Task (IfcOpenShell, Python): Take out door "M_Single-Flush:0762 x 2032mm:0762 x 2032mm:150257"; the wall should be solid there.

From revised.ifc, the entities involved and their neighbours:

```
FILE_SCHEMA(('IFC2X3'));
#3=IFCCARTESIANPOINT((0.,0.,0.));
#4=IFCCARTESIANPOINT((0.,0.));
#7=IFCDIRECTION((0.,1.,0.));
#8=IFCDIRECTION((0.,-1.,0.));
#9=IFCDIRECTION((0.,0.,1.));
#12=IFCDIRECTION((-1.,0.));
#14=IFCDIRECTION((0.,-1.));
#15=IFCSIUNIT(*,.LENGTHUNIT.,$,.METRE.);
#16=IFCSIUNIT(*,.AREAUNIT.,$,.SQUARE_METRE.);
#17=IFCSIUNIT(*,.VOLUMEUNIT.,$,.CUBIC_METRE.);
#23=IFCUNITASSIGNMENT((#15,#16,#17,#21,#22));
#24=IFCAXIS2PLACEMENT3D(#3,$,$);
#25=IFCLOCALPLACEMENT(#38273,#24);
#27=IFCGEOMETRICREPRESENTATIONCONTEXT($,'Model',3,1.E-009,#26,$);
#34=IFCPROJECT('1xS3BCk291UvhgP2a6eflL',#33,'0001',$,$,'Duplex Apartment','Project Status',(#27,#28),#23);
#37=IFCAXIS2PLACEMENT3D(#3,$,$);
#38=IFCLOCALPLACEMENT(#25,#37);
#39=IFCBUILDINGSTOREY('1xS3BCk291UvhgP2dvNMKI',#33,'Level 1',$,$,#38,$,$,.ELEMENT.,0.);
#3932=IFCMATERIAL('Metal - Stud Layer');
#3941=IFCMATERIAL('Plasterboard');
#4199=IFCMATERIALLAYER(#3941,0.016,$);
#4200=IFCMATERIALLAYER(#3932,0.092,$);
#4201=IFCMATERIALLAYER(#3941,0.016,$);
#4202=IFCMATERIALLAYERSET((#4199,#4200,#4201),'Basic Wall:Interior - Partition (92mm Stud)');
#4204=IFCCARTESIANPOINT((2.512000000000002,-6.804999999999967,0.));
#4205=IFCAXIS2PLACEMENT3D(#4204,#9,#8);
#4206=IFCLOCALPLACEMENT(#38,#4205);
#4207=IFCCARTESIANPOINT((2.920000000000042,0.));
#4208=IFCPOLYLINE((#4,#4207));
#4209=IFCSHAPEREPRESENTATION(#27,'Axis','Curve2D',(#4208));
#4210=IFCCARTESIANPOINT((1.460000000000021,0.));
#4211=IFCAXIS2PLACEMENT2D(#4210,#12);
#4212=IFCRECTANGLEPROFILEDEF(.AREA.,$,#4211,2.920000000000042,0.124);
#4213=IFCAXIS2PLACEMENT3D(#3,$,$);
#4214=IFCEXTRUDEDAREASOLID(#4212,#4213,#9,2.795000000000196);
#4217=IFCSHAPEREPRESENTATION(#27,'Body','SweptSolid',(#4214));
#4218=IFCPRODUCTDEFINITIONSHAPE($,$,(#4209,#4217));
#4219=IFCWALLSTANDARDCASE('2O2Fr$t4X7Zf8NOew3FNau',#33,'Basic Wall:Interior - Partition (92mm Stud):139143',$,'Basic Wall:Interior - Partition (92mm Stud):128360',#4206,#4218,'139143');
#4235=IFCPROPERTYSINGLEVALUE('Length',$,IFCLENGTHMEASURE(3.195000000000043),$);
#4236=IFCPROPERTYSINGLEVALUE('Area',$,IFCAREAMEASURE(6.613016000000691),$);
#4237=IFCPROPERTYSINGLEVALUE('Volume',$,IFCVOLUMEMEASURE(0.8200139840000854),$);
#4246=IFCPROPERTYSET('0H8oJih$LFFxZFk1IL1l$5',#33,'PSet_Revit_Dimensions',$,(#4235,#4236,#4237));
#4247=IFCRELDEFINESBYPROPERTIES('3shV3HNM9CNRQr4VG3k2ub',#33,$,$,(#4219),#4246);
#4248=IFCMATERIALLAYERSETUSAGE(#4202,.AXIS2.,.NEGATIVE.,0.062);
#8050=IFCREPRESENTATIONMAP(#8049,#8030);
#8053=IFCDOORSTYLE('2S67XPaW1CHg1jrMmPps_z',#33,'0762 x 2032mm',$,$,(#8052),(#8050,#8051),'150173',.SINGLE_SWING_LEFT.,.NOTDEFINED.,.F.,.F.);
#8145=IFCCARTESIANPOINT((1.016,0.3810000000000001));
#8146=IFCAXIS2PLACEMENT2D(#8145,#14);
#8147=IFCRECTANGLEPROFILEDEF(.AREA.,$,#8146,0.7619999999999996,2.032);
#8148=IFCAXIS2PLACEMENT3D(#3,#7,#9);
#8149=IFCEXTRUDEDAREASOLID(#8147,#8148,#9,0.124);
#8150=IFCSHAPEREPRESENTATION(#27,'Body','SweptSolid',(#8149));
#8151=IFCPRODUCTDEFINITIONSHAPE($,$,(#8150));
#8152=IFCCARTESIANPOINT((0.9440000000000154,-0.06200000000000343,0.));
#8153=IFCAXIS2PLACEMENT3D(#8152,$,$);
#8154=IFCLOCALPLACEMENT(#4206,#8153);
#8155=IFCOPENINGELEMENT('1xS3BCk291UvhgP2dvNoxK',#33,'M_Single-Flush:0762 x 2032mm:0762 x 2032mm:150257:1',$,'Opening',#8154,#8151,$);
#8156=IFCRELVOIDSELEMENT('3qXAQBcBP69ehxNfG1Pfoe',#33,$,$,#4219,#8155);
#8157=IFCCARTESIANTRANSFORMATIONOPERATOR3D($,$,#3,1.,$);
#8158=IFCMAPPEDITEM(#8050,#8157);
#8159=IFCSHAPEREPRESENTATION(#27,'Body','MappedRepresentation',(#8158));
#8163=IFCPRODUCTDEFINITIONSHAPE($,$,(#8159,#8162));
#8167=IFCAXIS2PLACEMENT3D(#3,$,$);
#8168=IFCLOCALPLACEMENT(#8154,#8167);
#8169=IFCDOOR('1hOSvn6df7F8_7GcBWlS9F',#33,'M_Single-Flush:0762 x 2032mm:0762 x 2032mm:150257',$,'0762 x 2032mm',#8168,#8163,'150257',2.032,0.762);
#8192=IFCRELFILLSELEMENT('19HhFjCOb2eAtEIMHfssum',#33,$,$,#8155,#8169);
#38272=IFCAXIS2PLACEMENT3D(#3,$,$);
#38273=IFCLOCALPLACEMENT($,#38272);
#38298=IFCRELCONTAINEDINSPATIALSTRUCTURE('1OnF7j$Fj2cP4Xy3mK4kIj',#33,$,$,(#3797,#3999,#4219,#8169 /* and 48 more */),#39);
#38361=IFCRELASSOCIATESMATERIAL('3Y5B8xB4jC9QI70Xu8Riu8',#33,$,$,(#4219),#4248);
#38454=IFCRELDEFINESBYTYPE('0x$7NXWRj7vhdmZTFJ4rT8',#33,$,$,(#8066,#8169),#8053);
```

```python
import ifcopenshell
import ifcopenshell.api.feature
import ifcopenshell.api.pset
import ifcopenshell.api.root
import ifcopenshell.geom
import ifcopenshell.util.element
import ifcopenshell.util.shape
import ifcopenshell.util.unit

model = ifcopenshell.open("revised.ifc")
area_scale = ifcopenshell.util.unit.calculate_unit_scale(model, "AREAUNIT")
volume_scale = ifcopenshell.util.unit.calculate_unit_scale(model, "VOLUMEUNIT")
settings = ifcopenshell.geom.settings()


def volume(element):
    """Net volume in cubic metres, openings subtracted."""
    shape = ifcopenshell.geom.create_shape(settings, element)
    return ifcopenshell.util.shape.get_volume(shape.geometry)


door = model.by_guid("1hOSvn6df7F8_7GcBWlS9F")
opening = door.FillsVoids[0].RelatingOpeningElement
wall = opening.VoidsElements[0].RelatingBuildingElement
before = volume(wall)

ifcopenshell.api.root.remove_product(model, product=door)
ifcopenshell.api.feature.remove_feature(model, feature=opening)

after = volume(wall)
thickness = 0.124  # wall thickness in metres

# Update the wall's stored quantities.
pset = model.by_id(ifcopenshell.util.element.get_pset(wall, "PSet_Revit_Dimensions", should_inherit=False)["id"])
ifcopenshell.api.pset.edit_pset(model, pset=pset, properties={
    "Area": model.create_entity("IfcAreaMeasure", after / thickness / area_scale),
    "Volume": model.create_entity("IfcVolumeMeasure", after / volume_scale),
})

print(f"wall volume {before:.3f} -> {after:.3f} m3")

model.write("revised-out.ifc")
```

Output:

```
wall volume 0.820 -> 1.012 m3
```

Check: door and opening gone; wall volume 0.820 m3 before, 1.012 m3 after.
